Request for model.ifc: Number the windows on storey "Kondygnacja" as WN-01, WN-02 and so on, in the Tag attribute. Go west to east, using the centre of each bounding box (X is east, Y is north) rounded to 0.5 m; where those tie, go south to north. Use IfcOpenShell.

First a look at what the model holds.

```python
import ifcopenshell
import ifcopenshell.util.element
import ifcopenshell.util.placement

model = ifcopenshell.open("model.ifc")
print(model.schema)
storey = next(s for s in model.by_type("IfcBuildingStorey") if s.Name == "Kondygnacja")
windows = [e for e in ifcopenshell.util.element.get_decomposition(storey) if e.is_a("IfcWindow")]
for e in sorted(windows, key=lambda e: e.id()):
    origin = ifcopenshell.util.placement.get_local_placement(e.ObjectPlacement)[:3, 3]
    print(e.id(), e.Tag, e.Name, origin.round(2) + 0.0, sep=" | ")
```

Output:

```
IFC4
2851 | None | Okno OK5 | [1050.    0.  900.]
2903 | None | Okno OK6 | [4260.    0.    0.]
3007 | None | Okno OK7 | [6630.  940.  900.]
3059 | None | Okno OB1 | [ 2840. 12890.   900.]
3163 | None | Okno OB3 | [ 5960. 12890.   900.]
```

```python
import ifcopenshell
import ifcopenshell.geom
import ifcopenshell.util.element
import ifcopenshell.util.shape

model = ifcopenshell.open("model.ifc")
settings = ifcopenshell.geom.settings()
settings.set("use-world-coords", True)


def centre(element):
    shape = ifcopenshell.geom.create_shape(settings, element)
    return ifcopenshell.util.shape.get_bbox_centroid(shape.geometry)


storey = next(s for s in model.by_type("IfcBuildingStorey") if s.Name == "Kondygnacja")
windows = [e for e in ifcopenshell.util.element.get_decomposition(storey) if e.is_a("IfcWindow")]

# Insertion points can sit at a corner or the storey origin, so sort by the geometry (in metres).
centres = {e: centre(e) for e in windows}
windows.sort(key=lambda e: (round(centres[e][0] / 0.5), centres[e][1]))

for i, e in enumerate(windows, start=1):
    number = f"WN-{i:02d}"
    e.Tag = number
    print(e.id(), number)

model.write("model_rev.ifc")
```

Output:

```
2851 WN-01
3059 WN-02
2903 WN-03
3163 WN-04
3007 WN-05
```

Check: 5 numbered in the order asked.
